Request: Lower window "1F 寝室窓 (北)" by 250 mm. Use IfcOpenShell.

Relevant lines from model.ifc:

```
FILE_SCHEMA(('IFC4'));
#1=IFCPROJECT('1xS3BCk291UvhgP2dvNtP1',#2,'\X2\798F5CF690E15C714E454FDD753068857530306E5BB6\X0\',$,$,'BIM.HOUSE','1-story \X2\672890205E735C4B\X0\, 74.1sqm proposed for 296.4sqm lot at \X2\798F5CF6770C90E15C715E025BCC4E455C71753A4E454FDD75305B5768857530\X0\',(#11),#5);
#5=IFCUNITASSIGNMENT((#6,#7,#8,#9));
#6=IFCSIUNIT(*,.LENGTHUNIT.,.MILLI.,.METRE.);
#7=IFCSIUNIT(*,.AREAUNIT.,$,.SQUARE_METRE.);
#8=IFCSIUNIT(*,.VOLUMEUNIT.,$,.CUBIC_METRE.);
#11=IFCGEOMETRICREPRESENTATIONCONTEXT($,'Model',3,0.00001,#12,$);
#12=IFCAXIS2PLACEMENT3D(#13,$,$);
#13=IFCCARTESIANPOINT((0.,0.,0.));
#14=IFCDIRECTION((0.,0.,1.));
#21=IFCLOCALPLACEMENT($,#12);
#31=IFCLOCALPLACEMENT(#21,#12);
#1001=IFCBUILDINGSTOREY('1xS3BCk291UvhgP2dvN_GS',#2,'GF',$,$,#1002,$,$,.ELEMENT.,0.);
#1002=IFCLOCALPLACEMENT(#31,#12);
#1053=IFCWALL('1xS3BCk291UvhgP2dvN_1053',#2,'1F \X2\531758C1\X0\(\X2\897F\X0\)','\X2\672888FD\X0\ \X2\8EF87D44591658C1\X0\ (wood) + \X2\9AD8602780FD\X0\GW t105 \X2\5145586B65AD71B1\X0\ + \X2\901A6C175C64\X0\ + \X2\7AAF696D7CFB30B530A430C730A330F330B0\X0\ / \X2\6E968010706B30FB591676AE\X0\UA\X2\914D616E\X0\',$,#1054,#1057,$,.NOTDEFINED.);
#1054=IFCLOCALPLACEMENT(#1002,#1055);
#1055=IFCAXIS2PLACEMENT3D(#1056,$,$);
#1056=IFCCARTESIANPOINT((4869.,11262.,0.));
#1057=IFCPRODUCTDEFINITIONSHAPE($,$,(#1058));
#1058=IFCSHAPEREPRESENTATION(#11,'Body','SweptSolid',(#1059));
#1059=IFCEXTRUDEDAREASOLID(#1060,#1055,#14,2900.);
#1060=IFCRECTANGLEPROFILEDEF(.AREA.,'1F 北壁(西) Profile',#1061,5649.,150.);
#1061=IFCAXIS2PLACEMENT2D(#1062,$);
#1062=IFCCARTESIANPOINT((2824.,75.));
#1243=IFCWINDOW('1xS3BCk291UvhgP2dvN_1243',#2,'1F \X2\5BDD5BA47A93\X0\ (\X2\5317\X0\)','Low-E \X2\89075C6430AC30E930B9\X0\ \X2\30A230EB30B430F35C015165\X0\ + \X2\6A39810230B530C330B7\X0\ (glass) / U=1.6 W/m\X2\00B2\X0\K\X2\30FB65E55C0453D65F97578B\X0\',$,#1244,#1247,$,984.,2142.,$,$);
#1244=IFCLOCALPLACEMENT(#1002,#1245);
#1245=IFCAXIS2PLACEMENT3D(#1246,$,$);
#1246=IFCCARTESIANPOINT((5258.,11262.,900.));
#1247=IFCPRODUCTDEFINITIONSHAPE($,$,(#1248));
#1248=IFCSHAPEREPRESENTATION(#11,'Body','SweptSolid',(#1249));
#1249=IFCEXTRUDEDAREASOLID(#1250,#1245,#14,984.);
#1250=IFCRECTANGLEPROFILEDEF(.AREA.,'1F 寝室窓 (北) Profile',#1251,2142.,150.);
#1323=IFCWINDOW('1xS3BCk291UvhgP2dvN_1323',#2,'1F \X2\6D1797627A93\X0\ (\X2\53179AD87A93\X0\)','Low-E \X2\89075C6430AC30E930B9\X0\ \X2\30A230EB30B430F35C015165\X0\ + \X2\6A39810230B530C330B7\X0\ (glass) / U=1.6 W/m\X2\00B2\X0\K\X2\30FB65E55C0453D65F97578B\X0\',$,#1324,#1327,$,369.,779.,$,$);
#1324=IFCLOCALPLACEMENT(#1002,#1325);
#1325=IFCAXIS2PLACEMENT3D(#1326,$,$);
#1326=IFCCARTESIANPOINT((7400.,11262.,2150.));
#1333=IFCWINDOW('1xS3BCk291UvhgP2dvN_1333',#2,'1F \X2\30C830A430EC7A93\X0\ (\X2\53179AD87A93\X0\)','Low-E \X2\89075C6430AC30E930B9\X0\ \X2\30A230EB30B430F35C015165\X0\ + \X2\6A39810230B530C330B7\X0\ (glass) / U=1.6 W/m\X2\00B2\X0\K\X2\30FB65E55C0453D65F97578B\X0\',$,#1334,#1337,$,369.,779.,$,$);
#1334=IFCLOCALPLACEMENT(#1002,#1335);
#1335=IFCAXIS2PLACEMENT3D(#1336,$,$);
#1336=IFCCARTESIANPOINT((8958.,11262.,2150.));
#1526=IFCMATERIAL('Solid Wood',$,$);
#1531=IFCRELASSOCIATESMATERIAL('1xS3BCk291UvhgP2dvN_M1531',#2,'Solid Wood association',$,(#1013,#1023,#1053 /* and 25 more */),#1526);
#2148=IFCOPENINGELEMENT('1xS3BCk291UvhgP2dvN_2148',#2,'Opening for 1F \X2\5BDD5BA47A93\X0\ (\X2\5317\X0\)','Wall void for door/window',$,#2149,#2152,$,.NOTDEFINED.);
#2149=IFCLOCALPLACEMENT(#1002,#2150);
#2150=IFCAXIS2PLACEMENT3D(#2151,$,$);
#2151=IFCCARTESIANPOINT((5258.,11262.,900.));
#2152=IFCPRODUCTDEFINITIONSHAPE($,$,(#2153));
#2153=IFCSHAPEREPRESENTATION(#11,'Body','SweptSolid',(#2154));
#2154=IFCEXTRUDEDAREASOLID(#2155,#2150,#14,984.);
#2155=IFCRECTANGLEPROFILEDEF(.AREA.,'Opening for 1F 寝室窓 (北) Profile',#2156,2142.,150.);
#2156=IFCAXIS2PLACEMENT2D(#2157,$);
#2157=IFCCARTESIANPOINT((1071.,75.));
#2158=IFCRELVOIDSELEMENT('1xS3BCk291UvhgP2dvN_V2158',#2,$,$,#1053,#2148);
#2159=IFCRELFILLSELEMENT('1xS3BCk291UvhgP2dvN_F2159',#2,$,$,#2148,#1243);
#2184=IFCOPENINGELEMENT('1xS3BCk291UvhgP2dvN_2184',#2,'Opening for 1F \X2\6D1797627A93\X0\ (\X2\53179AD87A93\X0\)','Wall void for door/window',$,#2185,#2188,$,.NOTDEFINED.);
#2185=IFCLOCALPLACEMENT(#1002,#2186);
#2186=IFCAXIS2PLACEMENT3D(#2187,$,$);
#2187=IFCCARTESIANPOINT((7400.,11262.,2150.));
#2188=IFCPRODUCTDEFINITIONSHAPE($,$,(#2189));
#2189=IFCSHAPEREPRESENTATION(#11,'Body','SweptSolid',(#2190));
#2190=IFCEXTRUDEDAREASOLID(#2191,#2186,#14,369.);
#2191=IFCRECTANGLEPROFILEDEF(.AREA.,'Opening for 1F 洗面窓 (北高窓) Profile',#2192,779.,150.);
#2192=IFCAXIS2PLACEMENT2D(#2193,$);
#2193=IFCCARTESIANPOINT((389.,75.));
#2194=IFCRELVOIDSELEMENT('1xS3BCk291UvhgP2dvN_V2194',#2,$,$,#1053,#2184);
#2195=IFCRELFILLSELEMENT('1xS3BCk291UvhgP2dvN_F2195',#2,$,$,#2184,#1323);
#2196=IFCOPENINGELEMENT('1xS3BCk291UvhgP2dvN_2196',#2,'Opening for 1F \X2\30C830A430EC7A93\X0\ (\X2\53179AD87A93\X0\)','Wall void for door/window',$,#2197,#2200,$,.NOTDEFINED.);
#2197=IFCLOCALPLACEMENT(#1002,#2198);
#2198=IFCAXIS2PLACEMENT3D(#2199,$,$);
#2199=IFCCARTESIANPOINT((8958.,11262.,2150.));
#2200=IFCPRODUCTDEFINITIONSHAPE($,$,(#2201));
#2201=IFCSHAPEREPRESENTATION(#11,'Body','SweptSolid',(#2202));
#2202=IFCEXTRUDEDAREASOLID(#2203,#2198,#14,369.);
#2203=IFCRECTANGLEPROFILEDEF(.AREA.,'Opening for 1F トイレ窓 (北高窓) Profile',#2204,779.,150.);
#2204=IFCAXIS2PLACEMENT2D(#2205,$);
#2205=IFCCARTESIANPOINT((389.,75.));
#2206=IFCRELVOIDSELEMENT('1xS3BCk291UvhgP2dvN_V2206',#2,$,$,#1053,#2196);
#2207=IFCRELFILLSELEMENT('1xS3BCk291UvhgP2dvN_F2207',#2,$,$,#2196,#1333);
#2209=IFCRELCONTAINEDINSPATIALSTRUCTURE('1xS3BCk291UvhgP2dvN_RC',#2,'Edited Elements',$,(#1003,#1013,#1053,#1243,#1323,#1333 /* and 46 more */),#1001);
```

```python
import numpy as np
import ifcopenshell
import ifcopenshell.api.geometry
import ifcopenshell.util.placement
import ifcopenshell.util.unit

model = ifcopenshell.open("model.ifc")
unit_scale = ifcopenshell.util.unit.calculate_unit_scale(model)

window = model.by_guid("1xS3BCk291UvhgP2dvN_1243")
opening = window.FillsVoids[0].RelatingOpeningElement
dz = -0.25 / unit_scale

shift = np.array([0.0, 0.0, dz])
# The window is not placed relative to its opening, so move both.
for product in (opening, window):
    matrix = ifcopenshell.util.placement.get_local_placement(product.ObjectPlacement)
    matrix[:3, 3] += shift
    ifcopenshell.api.geometry.edit_object_placement(model, product=product, matrix=matrix, is_si=False)

print(f"moved by {dz * unit_scale:+.3f} m")

model.write("model-out.ifc")
```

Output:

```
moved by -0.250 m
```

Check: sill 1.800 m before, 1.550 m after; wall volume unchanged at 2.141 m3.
